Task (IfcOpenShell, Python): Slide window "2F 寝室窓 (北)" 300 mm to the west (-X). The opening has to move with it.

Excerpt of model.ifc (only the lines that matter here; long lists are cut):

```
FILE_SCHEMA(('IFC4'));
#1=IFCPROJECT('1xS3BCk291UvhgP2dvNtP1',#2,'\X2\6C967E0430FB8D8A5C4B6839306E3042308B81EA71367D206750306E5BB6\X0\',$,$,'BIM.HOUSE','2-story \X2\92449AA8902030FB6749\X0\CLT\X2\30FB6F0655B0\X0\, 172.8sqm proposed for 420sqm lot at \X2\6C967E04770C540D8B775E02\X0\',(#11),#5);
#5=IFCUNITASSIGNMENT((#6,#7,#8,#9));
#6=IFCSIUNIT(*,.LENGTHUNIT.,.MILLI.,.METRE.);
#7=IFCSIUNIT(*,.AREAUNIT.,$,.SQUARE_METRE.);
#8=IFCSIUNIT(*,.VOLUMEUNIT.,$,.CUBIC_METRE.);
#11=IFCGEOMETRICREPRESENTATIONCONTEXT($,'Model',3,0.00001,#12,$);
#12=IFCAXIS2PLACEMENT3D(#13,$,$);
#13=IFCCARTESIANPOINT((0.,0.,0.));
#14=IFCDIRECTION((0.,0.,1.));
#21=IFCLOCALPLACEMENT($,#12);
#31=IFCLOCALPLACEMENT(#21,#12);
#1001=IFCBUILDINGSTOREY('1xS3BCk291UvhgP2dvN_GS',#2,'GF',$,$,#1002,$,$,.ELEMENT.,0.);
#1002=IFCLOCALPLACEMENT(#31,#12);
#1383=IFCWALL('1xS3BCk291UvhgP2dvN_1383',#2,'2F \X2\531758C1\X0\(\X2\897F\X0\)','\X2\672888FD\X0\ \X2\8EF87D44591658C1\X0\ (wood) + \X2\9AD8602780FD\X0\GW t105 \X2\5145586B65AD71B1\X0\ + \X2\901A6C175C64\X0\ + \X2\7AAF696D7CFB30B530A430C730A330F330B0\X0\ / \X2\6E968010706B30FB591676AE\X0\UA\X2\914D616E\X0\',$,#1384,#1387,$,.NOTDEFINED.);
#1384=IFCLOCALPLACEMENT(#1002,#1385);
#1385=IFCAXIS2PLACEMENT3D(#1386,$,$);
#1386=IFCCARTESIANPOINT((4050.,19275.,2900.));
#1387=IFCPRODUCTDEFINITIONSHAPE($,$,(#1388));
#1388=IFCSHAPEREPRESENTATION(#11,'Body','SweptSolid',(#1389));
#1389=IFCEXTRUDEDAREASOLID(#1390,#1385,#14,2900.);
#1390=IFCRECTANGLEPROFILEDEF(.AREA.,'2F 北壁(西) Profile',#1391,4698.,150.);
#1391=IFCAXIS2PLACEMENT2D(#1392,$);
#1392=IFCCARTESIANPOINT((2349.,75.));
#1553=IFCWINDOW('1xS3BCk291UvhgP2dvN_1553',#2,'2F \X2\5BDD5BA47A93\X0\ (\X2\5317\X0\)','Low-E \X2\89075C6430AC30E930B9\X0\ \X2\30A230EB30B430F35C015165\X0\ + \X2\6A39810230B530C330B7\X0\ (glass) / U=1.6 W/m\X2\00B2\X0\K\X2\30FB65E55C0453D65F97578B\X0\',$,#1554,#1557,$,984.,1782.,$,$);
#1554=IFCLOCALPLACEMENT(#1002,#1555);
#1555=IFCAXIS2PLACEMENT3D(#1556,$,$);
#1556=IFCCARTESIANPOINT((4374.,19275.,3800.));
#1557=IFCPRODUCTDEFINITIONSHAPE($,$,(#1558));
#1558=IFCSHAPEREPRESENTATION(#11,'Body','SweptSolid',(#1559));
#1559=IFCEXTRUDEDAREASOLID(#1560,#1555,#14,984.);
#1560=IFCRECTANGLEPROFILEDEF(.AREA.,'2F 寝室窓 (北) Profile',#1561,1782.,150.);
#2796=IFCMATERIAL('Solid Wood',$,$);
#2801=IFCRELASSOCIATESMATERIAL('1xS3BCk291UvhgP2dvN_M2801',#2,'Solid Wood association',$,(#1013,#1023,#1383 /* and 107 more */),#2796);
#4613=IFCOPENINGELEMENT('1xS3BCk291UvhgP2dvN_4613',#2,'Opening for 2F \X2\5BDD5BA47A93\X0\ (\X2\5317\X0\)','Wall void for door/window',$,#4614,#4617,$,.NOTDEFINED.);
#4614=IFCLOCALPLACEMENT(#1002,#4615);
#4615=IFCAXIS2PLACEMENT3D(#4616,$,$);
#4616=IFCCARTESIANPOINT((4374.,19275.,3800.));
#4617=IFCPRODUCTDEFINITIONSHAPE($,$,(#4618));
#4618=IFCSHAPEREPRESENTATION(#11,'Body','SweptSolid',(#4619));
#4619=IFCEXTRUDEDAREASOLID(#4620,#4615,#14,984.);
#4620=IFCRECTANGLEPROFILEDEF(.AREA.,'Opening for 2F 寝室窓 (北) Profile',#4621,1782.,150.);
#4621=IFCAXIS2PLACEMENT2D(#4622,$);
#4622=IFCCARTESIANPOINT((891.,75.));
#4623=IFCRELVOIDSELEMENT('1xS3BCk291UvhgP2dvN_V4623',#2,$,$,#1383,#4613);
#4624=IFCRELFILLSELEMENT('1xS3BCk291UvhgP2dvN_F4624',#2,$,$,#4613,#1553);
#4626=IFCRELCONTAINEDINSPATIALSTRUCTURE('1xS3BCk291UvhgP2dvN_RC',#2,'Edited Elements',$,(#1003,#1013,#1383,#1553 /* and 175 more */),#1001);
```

```python
import ifcopenshell
import ifcopenshell.api.geometry
import ifcopenshell.util.placement
import ifcopenshell.util.unit

model = ifcopenshell.open("model.ifc")
unit_scale = ifcopenshell.util.unit.calculate_unit_scale(model)

window = model.by_guid("1xS3BCk291UvhgP2dvN_1553")
opening = window.FillsVoids[0].RelatingOpeningElement
wall = opening.VoidsElements[0].RelatingBuildingElement

wall_matrix = ifcopenshell.util.placement.get_local_placement(wall.ObjectPlacement)
shift = wall_matrix[:3, 0] * -0.3 / unit_scale
before = ifcopenshell.util.placement.get_local_placement(window.ObjectPlacement)[:3, 3].copy()

# The window is not placed relative to its opening, so move both.
for product in (opening, window):
    matrix = ifcopenshell.util.placement.get_local_placement(product.ObjectPlacement)
    matrix[:3, 3] += shift
    ifcopenshell.api.geometry.edit_object_placement(model, product=product, matrix=matrix, is_si=False)

after = ifcopenshell.util.placement.get_local_placement(window.ObjectPlacement)[:3, 3]
print("window moved by", (after - before).round(3) + 0.0)

model.write("model_rev.ifc")
```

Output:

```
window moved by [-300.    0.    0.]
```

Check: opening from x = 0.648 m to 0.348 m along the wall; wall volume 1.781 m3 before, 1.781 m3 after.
